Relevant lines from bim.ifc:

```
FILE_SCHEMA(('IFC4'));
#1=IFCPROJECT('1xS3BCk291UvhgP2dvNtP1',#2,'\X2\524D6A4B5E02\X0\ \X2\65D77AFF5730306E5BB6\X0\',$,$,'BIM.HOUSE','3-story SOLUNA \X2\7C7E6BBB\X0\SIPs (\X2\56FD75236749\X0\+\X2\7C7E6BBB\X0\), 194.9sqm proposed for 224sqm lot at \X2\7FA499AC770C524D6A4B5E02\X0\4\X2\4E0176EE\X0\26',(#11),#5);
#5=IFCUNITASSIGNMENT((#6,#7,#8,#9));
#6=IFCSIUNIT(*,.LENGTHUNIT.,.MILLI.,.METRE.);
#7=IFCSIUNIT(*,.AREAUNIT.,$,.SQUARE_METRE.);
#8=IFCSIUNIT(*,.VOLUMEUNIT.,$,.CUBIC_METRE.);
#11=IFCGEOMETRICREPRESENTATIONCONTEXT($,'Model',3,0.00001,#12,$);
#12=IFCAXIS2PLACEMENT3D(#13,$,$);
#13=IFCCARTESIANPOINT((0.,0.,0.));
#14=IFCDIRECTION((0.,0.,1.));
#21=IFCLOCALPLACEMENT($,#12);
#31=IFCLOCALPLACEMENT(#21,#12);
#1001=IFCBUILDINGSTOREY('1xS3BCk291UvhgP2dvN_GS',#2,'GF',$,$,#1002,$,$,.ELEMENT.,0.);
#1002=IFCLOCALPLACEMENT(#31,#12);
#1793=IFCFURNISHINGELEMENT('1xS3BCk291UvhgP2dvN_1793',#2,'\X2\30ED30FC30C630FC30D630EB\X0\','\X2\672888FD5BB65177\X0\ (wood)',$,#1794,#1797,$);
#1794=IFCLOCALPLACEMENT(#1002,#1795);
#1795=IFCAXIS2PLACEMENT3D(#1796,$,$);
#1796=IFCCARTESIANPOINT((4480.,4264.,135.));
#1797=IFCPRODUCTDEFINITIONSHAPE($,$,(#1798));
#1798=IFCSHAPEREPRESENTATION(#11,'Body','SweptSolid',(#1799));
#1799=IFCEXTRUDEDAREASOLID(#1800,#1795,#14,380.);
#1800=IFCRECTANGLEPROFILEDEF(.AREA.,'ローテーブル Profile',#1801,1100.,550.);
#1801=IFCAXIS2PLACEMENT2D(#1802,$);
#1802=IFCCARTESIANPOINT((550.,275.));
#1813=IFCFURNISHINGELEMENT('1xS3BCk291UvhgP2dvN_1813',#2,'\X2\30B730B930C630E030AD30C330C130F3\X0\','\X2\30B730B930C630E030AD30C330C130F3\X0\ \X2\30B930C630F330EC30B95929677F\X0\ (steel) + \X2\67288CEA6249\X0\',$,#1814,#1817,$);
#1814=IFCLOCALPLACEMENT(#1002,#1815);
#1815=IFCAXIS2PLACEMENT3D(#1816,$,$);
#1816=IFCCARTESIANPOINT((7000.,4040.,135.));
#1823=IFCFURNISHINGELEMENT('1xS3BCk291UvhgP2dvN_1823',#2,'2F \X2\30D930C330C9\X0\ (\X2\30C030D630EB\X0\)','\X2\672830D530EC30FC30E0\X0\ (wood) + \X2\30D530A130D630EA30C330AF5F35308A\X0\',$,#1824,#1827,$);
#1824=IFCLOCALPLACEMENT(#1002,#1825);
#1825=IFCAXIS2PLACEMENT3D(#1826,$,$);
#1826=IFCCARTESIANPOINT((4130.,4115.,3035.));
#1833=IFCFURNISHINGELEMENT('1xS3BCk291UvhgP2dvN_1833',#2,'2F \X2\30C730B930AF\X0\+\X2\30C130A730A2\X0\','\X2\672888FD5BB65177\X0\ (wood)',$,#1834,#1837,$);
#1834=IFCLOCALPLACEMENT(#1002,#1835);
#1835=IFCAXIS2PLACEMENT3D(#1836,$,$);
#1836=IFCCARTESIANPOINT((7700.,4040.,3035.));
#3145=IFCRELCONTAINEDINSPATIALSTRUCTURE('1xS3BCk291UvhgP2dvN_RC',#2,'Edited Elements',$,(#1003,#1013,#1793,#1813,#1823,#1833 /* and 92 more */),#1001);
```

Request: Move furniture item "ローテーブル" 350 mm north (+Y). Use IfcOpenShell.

```python
import ifcopenshell
import ifcopenshell.api.geometry
import ifcopenshell.util.placement

model = ifcopenshell.open("bim.ifc")

item = model.by_guid("1xS3BCk291UvhgP2dvN_1793")
matrix = ifcopenshell.util.placement.get_local_placement(item.ObjectPlacement)
matrix[1, 3] += 350.0
ifcopenshell.api.geometry.edit_object_placement(model, product=item, matrix=matrix, is_si=False)

print(ifcopenshell.util.placement.get_local_placement(item.ObjectPlacement).round(3) + 0.0)

model.write("bim_updated.ifc")
```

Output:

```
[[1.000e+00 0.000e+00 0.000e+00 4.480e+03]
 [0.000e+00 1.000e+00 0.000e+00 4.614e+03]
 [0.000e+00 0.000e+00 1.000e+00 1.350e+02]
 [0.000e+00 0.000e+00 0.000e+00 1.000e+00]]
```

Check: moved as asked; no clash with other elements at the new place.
